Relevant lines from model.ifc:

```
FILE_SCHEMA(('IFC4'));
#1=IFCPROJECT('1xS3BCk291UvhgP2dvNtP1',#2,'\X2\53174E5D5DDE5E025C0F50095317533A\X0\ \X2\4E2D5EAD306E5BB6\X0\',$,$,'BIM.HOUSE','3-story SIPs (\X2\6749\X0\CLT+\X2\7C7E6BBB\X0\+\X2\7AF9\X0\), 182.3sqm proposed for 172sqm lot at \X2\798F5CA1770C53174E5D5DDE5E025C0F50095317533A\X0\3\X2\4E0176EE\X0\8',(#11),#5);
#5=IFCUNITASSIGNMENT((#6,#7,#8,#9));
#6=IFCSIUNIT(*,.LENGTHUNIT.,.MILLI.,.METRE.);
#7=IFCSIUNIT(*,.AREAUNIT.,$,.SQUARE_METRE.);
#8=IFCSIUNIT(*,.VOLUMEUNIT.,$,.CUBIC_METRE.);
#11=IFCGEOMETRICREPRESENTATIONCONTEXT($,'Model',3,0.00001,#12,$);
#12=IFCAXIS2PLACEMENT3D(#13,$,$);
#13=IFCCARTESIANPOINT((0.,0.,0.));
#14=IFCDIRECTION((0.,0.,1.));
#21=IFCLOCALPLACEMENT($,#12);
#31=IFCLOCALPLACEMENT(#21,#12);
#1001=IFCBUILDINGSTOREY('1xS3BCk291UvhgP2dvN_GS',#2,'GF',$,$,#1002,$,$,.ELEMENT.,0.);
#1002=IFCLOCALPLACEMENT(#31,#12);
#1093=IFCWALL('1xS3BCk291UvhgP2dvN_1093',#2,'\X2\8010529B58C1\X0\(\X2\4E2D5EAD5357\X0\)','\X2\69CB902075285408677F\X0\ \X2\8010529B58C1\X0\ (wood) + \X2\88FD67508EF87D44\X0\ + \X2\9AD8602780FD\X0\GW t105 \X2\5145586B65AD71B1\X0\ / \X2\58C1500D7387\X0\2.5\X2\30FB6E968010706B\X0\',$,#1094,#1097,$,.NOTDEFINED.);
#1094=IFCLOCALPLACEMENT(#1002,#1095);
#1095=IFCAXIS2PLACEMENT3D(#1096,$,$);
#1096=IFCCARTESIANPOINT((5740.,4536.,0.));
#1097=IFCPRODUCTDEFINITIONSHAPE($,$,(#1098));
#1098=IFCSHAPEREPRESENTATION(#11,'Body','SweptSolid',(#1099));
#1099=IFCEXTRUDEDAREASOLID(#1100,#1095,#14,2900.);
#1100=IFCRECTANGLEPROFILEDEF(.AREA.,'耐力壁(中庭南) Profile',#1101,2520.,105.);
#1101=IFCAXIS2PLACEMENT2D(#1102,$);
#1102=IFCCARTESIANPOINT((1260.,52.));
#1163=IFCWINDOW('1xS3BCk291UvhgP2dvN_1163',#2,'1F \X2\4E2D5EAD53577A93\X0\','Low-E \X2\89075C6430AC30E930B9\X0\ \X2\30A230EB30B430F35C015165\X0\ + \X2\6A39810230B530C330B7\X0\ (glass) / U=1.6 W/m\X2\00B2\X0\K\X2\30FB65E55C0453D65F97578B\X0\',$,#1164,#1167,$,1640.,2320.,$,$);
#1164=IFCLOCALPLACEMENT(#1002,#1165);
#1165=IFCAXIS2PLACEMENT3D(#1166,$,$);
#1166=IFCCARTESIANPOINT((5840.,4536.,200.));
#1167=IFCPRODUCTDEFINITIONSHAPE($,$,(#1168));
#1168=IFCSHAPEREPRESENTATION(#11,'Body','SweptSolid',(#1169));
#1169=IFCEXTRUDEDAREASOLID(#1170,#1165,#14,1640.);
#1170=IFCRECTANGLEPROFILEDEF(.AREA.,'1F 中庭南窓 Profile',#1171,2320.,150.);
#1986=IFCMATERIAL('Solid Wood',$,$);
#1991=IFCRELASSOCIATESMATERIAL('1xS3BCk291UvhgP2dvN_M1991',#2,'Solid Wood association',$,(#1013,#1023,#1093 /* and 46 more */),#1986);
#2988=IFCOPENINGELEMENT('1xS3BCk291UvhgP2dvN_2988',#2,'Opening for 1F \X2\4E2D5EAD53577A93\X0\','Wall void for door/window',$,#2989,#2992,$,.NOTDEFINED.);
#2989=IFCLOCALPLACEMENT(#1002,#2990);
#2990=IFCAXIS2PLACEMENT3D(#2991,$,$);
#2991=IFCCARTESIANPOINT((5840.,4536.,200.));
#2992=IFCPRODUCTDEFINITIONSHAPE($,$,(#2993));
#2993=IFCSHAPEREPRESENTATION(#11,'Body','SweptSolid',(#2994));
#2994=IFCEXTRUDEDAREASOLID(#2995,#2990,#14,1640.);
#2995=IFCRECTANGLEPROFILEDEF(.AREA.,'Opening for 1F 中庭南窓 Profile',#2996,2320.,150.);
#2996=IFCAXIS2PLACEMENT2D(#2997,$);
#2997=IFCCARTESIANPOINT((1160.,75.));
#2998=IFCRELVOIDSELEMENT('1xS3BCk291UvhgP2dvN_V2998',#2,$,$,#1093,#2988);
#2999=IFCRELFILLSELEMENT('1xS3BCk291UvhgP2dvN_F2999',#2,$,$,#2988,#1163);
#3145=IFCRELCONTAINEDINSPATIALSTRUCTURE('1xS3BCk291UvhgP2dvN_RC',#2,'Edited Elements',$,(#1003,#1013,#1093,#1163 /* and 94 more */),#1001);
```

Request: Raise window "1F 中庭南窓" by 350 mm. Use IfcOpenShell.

```python
import numpy as np
import ifcopenshell
import ifcopenshell.api.geometry
import ifcopenshell.util.placement
import ifcopenshell.util.unit

model = ifcopenshell.open("model.ifc")
unit_scale = ifcopenshell.util.unit.calculate_unit_scale(model)

window = model.by_guid("1xS3BCk291UvhgP2dvN_1163")
opening = window.FillsVoids[0].RelatingOpeningElement
dz = 0.35 / unit_scale

shift = np.array([0.0, 0.0, dz])
# The window is not placed relative to its opening, so move both.
for product in (opening, window):
    matrix = ifcopenshell.util.placement.get_local_placement(product.ObjectPlacement)
    matrix[:3, 3] += shift
    ifcopenshell.api.geometry.edit_object_placement(model, product=product, matrix=matrix, is_si=False)

print(f"moved by {dz * unit_scale:+.3f} m")

model.write("model-out.ifc")
```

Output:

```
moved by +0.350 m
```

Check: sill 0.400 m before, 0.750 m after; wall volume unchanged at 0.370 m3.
